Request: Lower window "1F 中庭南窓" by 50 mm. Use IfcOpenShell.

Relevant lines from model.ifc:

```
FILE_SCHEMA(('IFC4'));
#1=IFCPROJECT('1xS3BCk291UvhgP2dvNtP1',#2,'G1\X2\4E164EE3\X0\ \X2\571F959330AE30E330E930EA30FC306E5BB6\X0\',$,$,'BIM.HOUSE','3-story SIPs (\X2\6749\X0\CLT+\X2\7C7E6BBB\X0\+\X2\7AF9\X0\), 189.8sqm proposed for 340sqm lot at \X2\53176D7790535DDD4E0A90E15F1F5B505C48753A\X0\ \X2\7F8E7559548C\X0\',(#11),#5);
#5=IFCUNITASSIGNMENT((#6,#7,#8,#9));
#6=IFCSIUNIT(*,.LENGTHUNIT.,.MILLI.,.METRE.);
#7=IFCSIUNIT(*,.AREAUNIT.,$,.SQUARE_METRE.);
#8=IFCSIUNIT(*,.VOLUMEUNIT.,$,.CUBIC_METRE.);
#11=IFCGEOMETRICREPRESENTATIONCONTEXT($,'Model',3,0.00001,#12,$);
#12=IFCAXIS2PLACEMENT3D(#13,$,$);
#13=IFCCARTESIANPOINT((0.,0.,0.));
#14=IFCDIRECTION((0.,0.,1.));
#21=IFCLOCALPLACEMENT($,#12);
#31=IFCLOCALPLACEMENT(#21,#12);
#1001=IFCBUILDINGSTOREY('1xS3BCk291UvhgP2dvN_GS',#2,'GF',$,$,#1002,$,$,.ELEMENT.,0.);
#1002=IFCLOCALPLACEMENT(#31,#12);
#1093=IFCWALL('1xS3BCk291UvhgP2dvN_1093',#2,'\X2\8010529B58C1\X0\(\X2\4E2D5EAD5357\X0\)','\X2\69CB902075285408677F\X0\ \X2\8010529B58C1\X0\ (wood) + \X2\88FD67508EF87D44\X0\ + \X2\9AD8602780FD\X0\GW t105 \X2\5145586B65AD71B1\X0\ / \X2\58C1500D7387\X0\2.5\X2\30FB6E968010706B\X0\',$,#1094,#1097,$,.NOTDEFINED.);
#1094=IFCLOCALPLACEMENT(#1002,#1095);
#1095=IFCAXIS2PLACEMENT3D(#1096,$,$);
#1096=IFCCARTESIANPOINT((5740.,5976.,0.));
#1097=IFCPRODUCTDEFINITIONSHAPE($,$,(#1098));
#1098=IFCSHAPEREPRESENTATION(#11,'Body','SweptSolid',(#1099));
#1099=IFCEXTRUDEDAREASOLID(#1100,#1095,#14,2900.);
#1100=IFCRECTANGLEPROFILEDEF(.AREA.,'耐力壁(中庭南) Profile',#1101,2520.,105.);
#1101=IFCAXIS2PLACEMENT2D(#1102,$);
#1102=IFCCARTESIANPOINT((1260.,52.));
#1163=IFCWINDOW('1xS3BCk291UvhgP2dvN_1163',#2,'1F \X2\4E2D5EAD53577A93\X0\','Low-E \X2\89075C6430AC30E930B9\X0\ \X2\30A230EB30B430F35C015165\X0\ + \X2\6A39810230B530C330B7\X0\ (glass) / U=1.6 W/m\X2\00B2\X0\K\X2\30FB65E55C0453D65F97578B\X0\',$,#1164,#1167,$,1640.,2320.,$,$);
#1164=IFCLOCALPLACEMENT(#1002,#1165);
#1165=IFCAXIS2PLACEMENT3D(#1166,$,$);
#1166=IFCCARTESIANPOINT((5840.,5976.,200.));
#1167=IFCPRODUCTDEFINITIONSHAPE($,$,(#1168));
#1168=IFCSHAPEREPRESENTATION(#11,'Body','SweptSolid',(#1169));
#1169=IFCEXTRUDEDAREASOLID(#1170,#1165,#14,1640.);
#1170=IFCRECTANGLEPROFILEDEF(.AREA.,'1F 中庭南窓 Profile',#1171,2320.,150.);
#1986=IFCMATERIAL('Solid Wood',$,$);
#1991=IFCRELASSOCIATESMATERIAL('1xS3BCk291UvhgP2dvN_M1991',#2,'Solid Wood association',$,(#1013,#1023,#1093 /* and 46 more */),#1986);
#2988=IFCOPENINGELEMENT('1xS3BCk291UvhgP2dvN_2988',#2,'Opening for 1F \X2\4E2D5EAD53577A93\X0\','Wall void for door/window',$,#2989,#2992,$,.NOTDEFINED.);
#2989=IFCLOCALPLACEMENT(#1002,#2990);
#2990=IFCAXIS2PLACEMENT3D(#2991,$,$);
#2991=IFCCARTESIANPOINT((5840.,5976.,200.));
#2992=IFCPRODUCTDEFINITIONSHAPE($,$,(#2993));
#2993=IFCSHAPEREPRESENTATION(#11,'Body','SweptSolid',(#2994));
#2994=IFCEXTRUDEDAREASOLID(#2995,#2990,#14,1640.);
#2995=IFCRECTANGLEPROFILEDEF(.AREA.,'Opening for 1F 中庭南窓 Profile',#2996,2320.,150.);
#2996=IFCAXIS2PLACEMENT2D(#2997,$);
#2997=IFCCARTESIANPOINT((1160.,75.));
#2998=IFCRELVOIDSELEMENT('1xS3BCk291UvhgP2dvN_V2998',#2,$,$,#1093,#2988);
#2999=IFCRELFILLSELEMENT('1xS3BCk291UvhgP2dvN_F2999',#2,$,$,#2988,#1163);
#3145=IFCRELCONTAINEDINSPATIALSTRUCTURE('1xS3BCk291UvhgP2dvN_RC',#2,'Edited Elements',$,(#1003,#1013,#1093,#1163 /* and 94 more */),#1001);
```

```python
import numpy as np
import ifcopenshell
import ifcopenshell.api.geometry
import ifcopenshell.util.placement
import ifcopenshell.util.unit

model = ifcopenshell.open("model.ifc")
unit_scale = ifcopenshell.util.unit.calculate_unit_scale(model)

window = model.by_guid("1xS3BCk291UvhgP2dvN_1163")
opening = window.FillsVoids[0].RelatingOpeningElement
dz = -0.05 / unit_scale

shift = np.array([0.0, 0.0, dz])
# The window is not placed relative to its opening, so move both.
for product in (opening, window):
    matrix = ifcopenshell.util.placement.get_local_placement(product.ObjectPlacement)
    matrix[:3, 3] += shift
    ifcopenshell.api.geometry.edit_object_placement(model, product=product, matrix=matrix, is_si=False)

print(f"moved by {dz * unit_scale:+.3f} m")

model.write("model-out.ifc")
```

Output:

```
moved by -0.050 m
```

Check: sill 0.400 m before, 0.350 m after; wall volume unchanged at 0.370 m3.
